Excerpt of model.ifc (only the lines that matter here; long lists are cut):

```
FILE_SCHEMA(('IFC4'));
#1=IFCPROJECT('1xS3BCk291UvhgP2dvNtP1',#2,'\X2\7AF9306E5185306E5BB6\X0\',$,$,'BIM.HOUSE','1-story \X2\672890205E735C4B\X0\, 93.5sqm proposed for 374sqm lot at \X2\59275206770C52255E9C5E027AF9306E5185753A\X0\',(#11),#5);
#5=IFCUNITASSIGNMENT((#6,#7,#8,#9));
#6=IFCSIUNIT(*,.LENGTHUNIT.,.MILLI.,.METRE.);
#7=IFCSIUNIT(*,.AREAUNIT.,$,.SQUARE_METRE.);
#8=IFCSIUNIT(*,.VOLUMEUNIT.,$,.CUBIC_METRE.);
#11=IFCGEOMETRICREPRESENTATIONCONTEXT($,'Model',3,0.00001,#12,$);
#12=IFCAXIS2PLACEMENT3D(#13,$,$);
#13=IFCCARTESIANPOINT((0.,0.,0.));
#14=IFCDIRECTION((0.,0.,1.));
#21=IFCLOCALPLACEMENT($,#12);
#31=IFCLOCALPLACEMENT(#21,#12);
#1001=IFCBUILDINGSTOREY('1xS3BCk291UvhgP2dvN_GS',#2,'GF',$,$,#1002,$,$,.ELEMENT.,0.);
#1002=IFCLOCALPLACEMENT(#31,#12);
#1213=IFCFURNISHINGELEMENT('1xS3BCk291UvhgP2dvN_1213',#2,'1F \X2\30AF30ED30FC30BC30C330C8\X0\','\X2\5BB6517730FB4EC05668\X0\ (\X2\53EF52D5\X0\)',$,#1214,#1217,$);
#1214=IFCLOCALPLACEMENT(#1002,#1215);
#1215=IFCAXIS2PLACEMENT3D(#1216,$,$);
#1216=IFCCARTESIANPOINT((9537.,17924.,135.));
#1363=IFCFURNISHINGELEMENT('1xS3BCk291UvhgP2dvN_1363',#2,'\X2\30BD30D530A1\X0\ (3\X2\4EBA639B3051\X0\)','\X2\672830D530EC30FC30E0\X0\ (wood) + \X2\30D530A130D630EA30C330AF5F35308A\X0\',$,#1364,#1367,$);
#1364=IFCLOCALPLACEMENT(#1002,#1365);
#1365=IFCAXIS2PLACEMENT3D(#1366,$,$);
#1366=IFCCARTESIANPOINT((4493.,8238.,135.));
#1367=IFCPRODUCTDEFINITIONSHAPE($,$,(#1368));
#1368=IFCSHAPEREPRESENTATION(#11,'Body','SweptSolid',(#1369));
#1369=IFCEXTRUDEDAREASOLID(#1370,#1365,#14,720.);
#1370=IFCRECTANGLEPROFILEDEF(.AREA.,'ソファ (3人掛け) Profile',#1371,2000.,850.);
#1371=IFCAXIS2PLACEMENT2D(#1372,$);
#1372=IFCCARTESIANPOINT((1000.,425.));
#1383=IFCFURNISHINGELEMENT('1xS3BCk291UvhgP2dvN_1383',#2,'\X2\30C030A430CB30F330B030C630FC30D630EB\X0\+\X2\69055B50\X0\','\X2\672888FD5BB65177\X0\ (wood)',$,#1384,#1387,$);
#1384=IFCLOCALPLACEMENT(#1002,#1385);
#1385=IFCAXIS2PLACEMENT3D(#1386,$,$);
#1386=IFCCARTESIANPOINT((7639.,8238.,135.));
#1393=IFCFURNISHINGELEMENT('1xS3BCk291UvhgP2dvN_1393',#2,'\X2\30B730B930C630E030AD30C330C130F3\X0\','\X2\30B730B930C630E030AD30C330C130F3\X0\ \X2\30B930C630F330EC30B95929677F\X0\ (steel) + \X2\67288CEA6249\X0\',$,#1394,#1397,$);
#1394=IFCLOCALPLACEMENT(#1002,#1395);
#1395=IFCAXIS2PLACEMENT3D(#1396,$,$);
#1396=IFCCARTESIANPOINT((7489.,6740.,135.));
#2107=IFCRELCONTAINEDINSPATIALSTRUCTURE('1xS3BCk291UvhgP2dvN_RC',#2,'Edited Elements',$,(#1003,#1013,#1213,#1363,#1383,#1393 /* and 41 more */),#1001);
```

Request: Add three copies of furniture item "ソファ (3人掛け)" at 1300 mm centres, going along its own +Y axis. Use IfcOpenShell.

```python
import ifcopenshell
import ifcopenshell.api.geometry
import ifcopenshell.api.root
import ifcopenshell.util.element
import ifcopenshell.util.placement

model = ifcopenshell.open("model.ifc")


def reuse_history(source, copy):
    """copy_class also copies each property set's owner history, people and application; keep the originals."""
    for rel in copy.IsDefinedBy:
        if rel.is_a("IfcRelDefinesByProperties") and (history := rel.RelatingPropertyDefinition.OwnerHistory):
            rel.RelatingPropertyDefinition.OwnerHistory = source.OwnerHistory
            ifcopenshell.util.element.remove_deep2(model, history)


source = model.by_id(1363)
base = ifcopenshell.util.placement.get_local_placement(source.ObjectPlacement)
step = base[:3, 1] * 1300.0

for i in range(1, 4):
    copy = ifcopenshell.api.root.copy_class(model, product=source)
    copy.Representation = ifcopenshell.util.element.copy_deep(
        model, source.Representation, exclude=["IfcGeometricRepresentationContext", "IfcRepresentationMap"]
    )
    reuse_history(source, copy)
    matrix = base.copy()
    matrix[:3, 3] += i * step
    print("added at", matrix[:3, 3].round(3) + 0.0)
    ifcopenshell.api.geometry.edit_object_placement(model, product=copy, matrix=matrix, is_si=False)

model.write("model-out.ifc")
```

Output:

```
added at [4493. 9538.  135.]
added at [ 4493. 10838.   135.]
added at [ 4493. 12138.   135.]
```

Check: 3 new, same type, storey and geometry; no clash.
